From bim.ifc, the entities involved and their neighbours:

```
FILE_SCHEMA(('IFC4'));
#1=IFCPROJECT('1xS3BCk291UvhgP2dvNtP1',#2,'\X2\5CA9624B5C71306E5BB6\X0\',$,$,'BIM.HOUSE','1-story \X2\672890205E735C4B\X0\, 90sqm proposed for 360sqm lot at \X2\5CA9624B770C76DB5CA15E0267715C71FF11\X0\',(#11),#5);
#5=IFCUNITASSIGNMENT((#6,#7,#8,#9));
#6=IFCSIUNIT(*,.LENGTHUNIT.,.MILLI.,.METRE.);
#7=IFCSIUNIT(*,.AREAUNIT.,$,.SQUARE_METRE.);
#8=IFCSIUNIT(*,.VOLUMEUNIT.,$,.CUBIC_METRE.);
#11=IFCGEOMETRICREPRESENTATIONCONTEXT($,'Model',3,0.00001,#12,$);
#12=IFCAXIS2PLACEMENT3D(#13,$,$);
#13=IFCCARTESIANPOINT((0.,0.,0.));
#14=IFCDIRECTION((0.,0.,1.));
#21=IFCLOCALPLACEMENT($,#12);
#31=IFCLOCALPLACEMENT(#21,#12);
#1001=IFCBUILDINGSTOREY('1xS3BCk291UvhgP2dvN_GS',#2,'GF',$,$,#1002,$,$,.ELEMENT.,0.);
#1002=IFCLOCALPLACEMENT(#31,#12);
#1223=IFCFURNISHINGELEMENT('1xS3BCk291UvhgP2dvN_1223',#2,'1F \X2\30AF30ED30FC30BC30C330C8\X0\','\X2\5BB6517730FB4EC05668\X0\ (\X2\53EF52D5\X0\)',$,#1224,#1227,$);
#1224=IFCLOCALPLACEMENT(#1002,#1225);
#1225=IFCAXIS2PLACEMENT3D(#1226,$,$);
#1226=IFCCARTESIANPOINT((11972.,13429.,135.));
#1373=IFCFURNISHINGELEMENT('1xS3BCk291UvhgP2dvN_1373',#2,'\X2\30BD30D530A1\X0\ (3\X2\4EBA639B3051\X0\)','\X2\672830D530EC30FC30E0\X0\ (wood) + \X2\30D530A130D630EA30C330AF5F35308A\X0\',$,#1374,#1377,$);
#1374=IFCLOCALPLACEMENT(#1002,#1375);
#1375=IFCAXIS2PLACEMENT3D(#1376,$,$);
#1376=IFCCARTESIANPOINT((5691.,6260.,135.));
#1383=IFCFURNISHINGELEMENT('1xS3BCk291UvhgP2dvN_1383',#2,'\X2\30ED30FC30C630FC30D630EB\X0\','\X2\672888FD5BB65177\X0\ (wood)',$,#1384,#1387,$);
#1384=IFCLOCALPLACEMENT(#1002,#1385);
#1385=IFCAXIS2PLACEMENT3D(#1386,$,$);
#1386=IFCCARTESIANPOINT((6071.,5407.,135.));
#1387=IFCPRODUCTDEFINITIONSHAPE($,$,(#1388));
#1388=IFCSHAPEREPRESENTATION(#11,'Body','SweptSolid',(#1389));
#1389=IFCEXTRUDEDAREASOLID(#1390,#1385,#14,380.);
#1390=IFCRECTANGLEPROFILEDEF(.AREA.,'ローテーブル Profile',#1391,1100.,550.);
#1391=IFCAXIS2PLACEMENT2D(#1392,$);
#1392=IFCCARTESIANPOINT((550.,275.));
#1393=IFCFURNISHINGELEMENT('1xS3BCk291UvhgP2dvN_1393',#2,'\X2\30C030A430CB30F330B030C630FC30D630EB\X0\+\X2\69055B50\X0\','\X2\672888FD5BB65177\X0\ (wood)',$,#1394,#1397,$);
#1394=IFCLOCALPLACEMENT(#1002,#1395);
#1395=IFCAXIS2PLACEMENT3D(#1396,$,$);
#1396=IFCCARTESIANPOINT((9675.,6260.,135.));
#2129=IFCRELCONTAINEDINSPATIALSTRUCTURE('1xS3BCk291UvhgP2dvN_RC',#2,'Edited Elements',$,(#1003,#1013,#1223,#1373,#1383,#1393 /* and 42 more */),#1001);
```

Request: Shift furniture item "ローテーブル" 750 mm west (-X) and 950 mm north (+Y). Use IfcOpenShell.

```python
import ifcopenshell
import ifcopenshell.api.geometry
import ifcopenshell.util.placement
import ifcopenshell.util.unit

model = ifcopenshell.open("bim.ifc")
unit_scale = ifcopenshell.util.unit.calculate_unit_scale(model)

item = model.by_guid("1xS3BCk291UvhgP2dvN_1383")
matrix = ifcopenshell.util.placement.get_local_placement(item.ObjectPlacement)
matrix[0, 3] -= 0.75 / unit_scale
matrix[1, 3] += 0.95 / unit_scale
ifcopenshell.api.geometry.edit_object_placement(model, product=item, matrix=matrix, is_si=False)

print(ifcopenshell.util.placement.get_local_placement(item.ObjectPlacement).round(3) + 0.0)

model.write("bim_edited.ifc")
```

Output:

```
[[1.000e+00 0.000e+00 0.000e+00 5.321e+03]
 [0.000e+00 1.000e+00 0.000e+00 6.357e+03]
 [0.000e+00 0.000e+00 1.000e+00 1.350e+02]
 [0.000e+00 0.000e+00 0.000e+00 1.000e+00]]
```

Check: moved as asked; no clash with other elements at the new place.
